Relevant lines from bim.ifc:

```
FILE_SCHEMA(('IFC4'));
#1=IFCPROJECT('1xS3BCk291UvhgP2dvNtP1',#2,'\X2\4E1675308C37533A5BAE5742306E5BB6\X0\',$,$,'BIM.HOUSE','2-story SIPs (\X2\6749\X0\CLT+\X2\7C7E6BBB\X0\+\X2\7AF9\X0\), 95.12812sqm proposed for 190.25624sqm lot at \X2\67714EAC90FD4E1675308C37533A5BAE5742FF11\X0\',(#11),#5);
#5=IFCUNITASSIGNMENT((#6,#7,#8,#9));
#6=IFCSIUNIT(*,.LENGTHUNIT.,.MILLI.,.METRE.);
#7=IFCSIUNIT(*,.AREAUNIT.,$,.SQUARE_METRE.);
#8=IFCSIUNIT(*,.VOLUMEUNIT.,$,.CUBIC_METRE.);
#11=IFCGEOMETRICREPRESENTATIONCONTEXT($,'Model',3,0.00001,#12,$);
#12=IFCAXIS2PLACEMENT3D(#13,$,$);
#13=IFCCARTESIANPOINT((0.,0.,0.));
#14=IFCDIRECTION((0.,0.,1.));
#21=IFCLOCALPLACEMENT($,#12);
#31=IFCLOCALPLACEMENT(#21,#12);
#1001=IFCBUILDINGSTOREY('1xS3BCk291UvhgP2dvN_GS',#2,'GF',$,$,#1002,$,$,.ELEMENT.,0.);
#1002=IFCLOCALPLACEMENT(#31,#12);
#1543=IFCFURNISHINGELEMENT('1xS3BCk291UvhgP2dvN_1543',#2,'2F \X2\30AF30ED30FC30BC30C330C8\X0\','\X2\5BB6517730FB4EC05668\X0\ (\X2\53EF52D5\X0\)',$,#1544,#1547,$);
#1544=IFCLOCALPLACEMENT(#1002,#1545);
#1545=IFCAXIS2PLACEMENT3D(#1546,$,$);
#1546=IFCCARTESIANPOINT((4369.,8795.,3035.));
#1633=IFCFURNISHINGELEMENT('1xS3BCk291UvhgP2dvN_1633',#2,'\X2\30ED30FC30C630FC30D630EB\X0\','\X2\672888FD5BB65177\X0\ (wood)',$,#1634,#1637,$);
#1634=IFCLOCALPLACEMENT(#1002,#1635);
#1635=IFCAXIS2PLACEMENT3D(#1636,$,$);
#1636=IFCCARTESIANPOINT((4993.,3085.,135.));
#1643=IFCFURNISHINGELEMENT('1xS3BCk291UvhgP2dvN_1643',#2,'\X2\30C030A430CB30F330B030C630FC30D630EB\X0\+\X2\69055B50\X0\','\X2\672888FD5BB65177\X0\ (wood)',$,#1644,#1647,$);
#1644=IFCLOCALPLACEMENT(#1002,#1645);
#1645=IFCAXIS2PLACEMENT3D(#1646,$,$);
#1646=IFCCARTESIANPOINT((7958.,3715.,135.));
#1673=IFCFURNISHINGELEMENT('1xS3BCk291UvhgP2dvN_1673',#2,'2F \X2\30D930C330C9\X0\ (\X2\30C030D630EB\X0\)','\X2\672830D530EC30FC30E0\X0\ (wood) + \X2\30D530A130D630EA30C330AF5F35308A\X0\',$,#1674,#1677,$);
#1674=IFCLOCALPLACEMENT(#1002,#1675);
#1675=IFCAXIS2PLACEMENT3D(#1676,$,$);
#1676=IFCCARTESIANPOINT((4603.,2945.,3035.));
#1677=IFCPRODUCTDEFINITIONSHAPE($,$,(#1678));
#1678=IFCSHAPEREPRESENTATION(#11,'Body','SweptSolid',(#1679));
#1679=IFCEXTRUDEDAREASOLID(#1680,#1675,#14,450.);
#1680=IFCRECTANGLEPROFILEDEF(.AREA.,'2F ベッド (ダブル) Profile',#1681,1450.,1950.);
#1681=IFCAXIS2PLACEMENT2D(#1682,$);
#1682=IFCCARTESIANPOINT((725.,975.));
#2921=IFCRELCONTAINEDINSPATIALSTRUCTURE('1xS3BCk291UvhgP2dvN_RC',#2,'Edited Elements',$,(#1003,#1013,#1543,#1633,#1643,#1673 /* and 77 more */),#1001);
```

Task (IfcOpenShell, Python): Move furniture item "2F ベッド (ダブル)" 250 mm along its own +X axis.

```python
import ifcopenshell
import ifcopenshell.api.geometry
import ifcopenshell.util.placement
import ifcopenshell.util.unit

model = ifcopenshell.open("bim.ifc")
unit_scale = ifcopenshell.util.unit.calculate_unit_scale(model)

item = model.by_guid("1xS3BCk291UvhgP2dvN_1673")
matrix = ifcopenshell.util.placement.get_local_placement(item.ObjectPlacement)
matrix[:3, 3] += matrix[:3, 0] * 0.25 / unit_scale
ifcopenshell.api.geometry.edit_object_placement(model, product=item, matrix=matrix, is_si=False)

print(ifcopenshell.util.placement.get_local_placement(item.ObjectPlacement).round(3) + 0.0)

model.write("bim_rev.ifc")
```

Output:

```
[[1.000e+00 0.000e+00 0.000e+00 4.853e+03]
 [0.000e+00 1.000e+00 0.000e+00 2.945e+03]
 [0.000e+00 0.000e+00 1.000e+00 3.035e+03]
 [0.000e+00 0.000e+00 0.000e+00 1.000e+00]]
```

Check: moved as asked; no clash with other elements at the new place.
